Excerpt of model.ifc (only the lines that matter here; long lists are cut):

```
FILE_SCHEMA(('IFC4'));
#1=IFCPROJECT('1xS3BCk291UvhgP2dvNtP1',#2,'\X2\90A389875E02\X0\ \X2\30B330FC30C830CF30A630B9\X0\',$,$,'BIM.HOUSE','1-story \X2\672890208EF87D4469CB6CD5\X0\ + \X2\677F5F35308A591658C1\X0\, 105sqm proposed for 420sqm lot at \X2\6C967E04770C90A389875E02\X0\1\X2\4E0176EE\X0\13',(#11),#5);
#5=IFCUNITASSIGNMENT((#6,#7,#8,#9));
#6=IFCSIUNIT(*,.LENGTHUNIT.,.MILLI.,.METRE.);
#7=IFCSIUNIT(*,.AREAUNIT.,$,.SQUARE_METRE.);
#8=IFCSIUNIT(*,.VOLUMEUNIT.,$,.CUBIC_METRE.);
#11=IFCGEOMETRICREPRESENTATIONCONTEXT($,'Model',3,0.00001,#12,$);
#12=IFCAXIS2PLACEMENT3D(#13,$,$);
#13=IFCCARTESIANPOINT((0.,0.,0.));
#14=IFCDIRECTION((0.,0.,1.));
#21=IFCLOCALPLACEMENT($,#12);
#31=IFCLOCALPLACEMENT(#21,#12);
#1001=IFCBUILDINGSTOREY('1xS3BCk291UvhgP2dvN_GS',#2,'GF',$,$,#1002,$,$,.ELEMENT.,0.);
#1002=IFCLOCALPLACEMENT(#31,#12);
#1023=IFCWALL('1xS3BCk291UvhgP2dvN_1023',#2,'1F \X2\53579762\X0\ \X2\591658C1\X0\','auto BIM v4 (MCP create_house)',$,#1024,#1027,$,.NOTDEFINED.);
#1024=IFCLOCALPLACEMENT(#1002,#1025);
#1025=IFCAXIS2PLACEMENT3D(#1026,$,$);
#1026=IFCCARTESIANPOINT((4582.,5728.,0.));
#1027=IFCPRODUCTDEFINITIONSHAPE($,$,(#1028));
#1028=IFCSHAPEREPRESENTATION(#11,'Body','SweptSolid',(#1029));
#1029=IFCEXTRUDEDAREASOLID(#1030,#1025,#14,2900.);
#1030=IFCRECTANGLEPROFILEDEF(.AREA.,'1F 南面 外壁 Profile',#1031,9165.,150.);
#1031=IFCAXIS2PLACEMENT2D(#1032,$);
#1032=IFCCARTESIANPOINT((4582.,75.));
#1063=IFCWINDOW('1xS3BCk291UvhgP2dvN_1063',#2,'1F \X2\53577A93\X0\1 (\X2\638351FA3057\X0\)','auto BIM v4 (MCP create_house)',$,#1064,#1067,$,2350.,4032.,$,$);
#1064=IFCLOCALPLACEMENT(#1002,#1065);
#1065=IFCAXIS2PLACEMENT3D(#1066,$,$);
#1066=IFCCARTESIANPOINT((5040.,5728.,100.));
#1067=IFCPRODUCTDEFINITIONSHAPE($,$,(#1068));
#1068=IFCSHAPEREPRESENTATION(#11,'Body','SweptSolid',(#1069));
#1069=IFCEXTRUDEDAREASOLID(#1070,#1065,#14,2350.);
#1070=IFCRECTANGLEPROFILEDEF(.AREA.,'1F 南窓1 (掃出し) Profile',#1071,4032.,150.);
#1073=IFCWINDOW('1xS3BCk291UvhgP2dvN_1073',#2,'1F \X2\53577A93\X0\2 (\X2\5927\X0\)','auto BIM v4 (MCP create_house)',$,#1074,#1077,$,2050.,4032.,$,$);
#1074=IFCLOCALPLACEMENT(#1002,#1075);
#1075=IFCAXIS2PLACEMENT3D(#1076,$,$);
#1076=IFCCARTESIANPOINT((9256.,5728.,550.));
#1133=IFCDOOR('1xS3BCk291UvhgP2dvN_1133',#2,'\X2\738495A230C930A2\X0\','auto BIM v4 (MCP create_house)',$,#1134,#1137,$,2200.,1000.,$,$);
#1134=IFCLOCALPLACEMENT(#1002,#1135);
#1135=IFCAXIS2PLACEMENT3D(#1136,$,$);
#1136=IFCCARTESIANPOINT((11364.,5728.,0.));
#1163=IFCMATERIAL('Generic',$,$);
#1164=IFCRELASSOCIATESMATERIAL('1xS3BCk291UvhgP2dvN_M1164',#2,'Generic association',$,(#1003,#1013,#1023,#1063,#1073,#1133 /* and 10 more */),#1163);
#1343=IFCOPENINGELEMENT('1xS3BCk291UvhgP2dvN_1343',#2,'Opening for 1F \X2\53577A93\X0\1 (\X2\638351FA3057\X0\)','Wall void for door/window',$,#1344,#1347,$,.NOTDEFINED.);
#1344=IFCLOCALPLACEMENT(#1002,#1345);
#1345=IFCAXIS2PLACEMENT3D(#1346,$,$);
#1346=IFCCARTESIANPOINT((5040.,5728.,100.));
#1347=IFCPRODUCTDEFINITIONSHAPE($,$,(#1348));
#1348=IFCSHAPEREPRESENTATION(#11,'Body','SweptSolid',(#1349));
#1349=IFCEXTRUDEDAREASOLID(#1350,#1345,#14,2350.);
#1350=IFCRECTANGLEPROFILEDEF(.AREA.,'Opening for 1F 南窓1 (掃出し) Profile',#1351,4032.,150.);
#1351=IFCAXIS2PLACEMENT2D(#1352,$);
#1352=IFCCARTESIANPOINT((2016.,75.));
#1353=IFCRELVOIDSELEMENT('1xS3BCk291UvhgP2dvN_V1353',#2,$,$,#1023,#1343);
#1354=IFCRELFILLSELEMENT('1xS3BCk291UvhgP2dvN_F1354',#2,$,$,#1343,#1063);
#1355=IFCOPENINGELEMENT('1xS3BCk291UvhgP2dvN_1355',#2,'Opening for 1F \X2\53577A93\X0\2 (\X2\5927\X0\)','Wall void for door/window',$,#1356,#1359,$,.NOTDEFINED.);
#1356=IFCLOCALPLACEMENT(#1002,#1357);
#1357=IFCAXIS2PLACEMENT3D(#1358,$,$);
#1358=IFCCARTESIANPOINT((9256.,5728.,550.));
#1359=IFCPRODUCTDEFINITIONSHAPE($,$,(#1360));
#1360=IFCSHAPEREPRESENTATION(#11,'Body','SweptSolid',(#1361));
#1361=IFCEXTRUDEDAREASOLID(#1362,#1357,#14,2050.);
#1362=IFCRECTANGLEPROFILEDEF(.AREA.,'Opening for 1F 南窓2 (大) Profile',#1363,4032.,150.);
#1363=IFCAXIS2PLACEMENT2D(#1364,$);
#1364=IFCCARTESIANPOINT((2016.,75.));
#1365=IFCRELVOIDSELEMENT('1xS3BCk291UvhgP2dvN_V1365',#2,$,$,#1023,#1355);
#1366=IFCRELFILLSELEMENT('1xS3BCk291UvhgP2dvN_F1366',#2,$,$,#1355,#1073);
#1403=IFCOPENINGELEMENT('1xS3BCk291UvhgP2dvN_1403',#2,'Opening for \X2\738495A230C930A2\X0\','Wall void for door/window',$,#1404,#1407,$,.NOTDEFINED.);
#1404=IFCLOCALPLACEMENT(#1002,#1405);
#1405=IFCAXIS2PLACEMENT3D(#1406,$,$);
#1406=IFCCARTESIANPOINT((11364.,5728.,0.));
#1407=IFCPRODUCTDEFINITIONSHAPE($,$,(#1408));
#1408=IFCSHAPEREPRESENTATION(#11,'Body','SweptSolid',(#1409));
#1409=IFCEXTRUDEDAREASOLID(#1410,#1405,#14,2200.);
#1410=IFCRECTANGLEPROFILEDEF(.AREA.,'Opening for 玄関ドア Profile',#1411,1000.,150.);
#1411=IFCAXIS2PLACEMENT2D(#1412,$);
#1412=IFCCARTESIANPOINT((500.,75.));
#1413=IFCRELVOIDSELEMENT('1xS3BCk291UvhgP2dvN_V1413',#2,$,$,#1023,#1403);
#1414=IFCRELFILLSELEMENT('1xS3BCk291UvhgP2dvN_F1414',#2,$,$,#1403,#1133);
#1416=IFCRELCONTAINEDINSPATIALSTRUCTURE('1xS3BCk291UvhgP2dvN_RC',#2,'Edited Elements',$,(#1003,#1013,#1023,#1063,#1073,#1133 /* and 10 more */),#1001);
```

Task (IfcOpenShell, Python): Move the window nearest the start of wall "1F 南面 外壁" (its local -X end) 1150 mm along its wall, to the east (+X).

```python
import ifcopenshell
import ifcopenshell.api.geometry
import ifcopenshell.util.placement
import ifcopenshell.util.unit

model = ifcopenshell.open("model.ifc")
unit_scale = ifcopenshell.util.unit.calculate_unit_scale(model)

window = model.by_id(1063)
opening = window.FillsVoids[0].RelatingOpeningElement
wall = opening.VoidsElements[0].RelatingBuildingElement

wall_matrix = ifcopenshell.util.placement.get_local_placement(wall.ObjectPlacement)
shift = wall_matrix[:3, 0] * 1.15 / unit_scale
before = ifcopenshell.util.placement.get_local_placement(window.ObjectPlacement)[:3, 3].copy()

# The window is not placed relative to its opening, so move both.
for product in (opening, window):
    matrix = ifcopenshell.util.placement.get_local_placement(product.ObjectPlacement)
    matrix[:3, 3] += shift
    ifcopenshell.api.geometry.edit_object_placement(model, product=product, matrix=matrix, is_si=False)

after = ifcopenshell.util.placement.get_local_placement(window.ObjectPlacement)[:3, 3]
print("window moved by", (after - before).round(3) + 0.0)

model.write("model-out.ifc")
```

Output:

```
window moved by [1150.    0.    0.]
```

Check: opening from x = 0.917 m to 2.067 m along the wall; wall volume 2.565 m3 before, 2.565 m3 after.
